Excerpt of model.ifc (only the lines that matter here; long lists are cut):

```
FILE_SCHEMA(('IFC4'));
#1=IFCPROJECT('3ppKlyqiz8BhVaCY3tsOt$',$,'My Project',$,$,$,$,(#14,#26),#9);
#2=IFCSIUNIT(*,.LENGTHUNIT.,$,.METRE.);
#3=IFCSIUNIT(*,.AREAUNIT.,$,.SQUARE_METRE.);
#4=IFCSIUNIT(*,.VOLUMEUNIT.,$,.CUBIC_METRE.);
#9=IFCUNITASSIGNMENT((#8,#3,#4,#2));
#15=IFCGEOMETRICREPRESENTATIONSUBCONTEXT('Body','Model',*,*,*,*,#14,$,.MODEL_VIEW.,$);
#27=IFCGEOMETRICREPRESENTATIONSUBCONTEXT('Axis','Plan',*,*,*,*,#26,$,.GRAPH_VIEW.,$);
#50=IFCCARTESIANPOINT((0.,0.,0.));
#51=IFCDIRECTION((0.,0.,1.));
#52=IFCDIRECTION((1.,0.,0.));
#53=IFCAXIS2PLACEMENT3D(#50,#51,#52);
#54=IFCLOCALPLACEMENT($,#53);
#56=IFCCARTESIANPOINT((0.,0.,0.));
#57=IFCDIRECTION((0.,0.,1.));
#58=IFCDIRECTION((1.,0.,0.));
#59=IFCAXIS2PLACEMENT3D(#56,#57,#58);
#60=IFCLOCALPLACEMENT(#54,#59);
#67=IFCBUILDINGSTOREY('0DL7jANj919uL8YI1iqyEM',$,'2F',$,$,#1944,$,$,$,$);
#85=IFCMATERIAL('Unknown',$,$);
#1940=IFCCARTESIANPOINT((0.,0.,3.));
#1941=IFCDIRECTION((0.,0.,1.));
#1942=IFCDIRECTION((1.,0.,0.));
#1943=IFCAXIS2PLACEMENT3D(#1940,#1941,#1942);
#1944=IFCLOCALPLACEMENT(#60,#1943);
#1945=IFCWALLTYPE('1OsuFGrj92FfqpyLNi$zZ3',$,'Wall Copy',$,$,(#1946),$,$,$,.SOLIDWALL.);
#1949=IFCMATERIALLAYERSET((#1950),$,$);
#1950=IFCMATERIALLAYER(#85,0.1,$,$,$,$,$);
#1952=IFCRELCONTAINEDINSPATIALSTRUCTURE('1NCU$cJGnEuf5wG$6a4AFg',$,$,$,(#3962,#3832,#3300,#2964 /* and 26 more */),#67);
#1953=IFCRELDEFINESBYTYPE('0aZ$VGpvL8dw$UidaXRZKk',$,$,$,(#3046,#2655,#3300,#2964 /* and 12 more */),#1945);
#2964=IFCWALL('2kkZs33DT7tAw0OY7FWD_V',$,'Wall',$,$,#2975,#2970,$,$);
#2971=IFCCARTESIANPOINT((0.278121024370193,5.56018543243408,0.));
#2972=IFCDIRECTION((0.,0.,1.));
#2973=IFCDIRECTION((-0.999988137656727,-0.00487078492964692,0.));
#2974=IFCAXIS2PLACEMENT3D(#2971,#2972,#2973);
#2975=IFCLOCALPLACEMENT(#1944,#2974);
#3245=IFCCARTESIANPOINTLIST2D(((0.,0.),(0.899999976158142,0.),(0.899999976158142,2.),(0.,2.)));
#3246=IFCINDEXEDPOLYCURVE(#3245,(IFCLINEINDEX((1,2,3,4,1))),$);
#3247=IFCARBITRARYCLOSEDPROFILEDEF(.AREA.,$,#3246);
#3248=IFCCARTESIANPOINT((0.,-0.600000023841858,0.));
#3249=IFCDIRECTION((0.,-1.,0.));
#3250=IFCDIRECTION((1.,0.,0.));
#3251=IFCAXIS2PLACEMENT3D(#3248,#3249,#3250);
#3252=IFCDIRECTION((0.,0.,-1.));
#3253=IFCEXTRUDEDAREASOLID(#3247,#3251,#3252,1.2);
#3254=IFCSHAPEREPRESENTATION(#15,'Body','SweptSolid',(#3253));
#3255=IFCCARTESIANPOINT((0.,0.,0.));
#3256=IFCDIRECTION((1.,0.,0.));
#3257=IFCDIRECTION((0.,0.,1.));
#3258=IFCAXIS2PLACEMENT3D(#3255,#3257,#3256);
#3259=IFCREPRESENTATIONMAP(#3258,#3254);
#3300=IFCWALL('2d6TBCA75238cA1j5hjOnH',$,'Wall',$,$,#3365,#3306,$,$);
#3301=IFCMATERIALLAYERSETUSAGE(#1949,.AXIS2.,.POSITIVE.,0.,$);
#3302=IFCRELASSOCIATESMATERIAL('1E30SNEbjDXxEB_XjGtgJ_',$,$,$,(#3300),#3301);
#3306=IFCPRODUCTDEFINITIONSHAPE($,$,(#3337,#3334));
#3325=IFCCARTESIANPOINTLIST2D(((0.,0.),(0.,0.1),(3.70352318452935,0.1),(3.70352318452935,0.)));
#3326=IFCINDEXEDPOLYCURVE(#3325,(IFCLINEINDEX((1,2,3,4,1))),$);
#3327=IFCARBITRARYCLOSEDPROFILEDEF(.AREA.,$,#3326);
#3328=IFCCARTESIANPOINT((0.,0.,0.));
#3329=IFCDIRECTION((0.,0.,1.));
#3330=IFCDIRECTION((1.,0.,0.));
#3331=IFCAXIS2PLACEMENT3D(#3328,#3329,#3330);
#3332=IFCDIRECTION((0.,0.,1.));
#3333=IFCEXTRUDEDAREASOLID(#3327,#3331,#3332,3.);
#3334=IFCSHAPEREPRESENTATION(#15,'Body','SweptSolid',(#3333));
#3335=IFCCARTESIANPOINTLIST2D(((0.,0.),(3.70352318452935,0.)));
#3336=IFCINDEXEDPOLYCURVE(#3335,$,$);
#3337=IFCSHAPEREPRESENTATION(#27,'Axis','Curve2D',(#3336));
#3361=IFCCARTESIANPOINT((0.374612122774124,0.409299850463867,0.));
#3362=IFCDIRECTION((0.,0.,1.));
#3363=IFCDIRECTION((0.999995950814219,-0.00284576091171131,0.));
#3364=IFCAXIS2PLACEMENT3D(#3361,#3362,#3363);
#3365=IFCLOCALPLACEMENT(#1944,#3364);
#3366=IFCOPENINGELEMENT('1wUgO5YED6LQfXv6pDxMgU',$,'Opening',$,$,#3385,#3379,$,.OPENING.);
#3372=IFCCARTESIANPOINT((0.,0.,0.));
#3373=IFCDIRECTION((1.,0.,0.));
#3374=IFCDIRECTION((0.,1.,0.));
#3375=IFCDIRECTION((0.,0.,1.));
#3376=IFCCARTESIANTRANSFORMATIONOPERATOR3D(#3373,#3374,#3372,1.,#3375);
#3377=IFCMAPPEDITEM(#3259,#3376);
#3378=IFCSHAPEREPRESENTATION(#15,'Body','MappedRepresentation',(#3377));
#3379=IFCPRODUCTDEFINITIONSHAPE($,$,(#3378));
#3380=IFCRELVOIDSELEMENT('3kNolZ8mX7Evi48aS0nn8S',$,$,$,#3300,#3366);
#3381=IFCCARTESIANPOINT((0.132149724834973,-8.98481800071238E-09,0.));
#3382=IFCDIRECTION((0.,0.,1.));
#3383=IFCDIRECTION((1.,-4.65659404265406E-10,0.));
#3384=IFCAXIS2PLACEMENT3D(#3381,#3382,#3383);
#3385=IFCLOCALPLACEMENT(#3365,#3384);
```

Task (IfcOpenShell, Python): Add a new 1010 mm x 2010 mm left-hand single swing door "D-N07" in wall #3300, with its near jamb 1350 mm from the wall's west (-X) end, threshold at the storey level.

```python
import numpy as np
import ifcopenshell
import ifcopenshell.api.feature
import ifcopenshell.api.geometry
import ifcopenshell.api.root
import ifcopenshell.api.spatial
import ifcopenshell.geom
import ifcopenshell.util.element
import ifcopenshell.util.placement
import ifcopenshell.util.representation
import ifcopenshell.util.shape
import ifcopenshell.util.unit

model = ifcopenshell.open("model.ifc")
unit_scale = ifcopenshell.util.unit.calculate_unit_scale(model)
settings = ifcopenshell.geom.settings()


def volume(element):
    """Net volume in cubic metres, openings subtracted."""
    shape = ifcopenshell.geom.create_shape(settings, element)
    return ifcopenshell.util.shape.get_volume(shape.geometry)


wall = model.by_guid("2d6TBCA75238cA1j5hjOnH")
storey = ifcopenshell.util.element.get_container(wall, ifc_class="IfcBuildingStorey")
context = ifcopenshell.util.representation.get_context(model, "Model", "Body", "MODEL_VIEW")
before = volume(wall)

width, height, from_end, sill = 1.01, 2.01, 1.35, 0.0  # metres

# The wall runs along its own X axis, and the end named is its -X end.
wall_shape = ifcopenshell.geom.create_shape(settings, wall)
x, y, z = ifcopenshell.util.shape.get_vertices(wall_shape.geometry).T
start = x.min() + from_end
face, thickness = float(y.min()), float(y.max() - y.min())
wall_matrix = ifcopenshell.util.placement.get_local_placement(wall.ObjectPlacement)
level = ifcopenshell.util.placement.get_local_placement(storey.ObjectPlacement)[2, 3]


def in_wall(x, y):
    """Placement at x, y metres in the wall's axes, at sill height."""
    matrix = wall_matrix.copy()
    matrix[:, 3] = wall_matrix @ np.array([x / unit_scale, y / unit_scale, 0.0, 1.0])
    matrix[2, 3] = level + sill / unit_scale
    return matrix


# Opening: a box that overshoots both wall faces by 50 mm.
opening = ifcopenshell.api.root.create_entity(model, ifc_class="IfcOpeningElement", predefined_type="OPENING")
box = ifcopenshell.api.geometry.add_wall_representation(
    model, context=context, length=width, height=height, thickness=thickness + 0.1
)
ifcopenshell.api.geometry.assign_representation(model, product=opening, representation=box)
ifcopenshell.api.geometry.edit_object_placement(model, product=opening, matrix=in_wall(start, face - 0.05), is_si=False)
ifcopenshell.api.feature.add_feature(model, feature=opening, element=wall)

door = ifcopenshell.api.root.create_entity(model, ifc_class="IfcDoor", name="D-N07", predefined_type="DOOR")
door.OverallWidth, door.OverallHeight = width / unit_scale, height / unit_scale
door.OperationType = "SINGLE_SWING_LEFT"
body = ifcopenshell.api.geometry.add_door_representation(
    model,
    context=context,
    overall_width=door.OverallWidth,
    overall_height=door.OverallHeight,
    operation_type="SINGLE_SWING_LEFT",
    lining_properties={"LiningDepth": thickness / unit_scale, "ThresholdDepth": thickness / unit_scale},
)
ifcopenshell.api.geometry.assign_representation(model, product=door, representation=body)
ifcopenshell.api.spatial.assign_container(model, products=[door], relating_structure=storey)
ifcopenshell.api.feature.add_filling(model, opening=opening, element=door)

# The lining spans the wall, so the door starts at the wall face.
ifcopenshell.api.geometry.edit_object_placement(model, product=door, matrix=in_wall(start, face), is_si=False)

after = volume(wall)

print(f"wall volume {before:.3f} -> {after:.3f} m3")

model.write("model_edited.ifc")
```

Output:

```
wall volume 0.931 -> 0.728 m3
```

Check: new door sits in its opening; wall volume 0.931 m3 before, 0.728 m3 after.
